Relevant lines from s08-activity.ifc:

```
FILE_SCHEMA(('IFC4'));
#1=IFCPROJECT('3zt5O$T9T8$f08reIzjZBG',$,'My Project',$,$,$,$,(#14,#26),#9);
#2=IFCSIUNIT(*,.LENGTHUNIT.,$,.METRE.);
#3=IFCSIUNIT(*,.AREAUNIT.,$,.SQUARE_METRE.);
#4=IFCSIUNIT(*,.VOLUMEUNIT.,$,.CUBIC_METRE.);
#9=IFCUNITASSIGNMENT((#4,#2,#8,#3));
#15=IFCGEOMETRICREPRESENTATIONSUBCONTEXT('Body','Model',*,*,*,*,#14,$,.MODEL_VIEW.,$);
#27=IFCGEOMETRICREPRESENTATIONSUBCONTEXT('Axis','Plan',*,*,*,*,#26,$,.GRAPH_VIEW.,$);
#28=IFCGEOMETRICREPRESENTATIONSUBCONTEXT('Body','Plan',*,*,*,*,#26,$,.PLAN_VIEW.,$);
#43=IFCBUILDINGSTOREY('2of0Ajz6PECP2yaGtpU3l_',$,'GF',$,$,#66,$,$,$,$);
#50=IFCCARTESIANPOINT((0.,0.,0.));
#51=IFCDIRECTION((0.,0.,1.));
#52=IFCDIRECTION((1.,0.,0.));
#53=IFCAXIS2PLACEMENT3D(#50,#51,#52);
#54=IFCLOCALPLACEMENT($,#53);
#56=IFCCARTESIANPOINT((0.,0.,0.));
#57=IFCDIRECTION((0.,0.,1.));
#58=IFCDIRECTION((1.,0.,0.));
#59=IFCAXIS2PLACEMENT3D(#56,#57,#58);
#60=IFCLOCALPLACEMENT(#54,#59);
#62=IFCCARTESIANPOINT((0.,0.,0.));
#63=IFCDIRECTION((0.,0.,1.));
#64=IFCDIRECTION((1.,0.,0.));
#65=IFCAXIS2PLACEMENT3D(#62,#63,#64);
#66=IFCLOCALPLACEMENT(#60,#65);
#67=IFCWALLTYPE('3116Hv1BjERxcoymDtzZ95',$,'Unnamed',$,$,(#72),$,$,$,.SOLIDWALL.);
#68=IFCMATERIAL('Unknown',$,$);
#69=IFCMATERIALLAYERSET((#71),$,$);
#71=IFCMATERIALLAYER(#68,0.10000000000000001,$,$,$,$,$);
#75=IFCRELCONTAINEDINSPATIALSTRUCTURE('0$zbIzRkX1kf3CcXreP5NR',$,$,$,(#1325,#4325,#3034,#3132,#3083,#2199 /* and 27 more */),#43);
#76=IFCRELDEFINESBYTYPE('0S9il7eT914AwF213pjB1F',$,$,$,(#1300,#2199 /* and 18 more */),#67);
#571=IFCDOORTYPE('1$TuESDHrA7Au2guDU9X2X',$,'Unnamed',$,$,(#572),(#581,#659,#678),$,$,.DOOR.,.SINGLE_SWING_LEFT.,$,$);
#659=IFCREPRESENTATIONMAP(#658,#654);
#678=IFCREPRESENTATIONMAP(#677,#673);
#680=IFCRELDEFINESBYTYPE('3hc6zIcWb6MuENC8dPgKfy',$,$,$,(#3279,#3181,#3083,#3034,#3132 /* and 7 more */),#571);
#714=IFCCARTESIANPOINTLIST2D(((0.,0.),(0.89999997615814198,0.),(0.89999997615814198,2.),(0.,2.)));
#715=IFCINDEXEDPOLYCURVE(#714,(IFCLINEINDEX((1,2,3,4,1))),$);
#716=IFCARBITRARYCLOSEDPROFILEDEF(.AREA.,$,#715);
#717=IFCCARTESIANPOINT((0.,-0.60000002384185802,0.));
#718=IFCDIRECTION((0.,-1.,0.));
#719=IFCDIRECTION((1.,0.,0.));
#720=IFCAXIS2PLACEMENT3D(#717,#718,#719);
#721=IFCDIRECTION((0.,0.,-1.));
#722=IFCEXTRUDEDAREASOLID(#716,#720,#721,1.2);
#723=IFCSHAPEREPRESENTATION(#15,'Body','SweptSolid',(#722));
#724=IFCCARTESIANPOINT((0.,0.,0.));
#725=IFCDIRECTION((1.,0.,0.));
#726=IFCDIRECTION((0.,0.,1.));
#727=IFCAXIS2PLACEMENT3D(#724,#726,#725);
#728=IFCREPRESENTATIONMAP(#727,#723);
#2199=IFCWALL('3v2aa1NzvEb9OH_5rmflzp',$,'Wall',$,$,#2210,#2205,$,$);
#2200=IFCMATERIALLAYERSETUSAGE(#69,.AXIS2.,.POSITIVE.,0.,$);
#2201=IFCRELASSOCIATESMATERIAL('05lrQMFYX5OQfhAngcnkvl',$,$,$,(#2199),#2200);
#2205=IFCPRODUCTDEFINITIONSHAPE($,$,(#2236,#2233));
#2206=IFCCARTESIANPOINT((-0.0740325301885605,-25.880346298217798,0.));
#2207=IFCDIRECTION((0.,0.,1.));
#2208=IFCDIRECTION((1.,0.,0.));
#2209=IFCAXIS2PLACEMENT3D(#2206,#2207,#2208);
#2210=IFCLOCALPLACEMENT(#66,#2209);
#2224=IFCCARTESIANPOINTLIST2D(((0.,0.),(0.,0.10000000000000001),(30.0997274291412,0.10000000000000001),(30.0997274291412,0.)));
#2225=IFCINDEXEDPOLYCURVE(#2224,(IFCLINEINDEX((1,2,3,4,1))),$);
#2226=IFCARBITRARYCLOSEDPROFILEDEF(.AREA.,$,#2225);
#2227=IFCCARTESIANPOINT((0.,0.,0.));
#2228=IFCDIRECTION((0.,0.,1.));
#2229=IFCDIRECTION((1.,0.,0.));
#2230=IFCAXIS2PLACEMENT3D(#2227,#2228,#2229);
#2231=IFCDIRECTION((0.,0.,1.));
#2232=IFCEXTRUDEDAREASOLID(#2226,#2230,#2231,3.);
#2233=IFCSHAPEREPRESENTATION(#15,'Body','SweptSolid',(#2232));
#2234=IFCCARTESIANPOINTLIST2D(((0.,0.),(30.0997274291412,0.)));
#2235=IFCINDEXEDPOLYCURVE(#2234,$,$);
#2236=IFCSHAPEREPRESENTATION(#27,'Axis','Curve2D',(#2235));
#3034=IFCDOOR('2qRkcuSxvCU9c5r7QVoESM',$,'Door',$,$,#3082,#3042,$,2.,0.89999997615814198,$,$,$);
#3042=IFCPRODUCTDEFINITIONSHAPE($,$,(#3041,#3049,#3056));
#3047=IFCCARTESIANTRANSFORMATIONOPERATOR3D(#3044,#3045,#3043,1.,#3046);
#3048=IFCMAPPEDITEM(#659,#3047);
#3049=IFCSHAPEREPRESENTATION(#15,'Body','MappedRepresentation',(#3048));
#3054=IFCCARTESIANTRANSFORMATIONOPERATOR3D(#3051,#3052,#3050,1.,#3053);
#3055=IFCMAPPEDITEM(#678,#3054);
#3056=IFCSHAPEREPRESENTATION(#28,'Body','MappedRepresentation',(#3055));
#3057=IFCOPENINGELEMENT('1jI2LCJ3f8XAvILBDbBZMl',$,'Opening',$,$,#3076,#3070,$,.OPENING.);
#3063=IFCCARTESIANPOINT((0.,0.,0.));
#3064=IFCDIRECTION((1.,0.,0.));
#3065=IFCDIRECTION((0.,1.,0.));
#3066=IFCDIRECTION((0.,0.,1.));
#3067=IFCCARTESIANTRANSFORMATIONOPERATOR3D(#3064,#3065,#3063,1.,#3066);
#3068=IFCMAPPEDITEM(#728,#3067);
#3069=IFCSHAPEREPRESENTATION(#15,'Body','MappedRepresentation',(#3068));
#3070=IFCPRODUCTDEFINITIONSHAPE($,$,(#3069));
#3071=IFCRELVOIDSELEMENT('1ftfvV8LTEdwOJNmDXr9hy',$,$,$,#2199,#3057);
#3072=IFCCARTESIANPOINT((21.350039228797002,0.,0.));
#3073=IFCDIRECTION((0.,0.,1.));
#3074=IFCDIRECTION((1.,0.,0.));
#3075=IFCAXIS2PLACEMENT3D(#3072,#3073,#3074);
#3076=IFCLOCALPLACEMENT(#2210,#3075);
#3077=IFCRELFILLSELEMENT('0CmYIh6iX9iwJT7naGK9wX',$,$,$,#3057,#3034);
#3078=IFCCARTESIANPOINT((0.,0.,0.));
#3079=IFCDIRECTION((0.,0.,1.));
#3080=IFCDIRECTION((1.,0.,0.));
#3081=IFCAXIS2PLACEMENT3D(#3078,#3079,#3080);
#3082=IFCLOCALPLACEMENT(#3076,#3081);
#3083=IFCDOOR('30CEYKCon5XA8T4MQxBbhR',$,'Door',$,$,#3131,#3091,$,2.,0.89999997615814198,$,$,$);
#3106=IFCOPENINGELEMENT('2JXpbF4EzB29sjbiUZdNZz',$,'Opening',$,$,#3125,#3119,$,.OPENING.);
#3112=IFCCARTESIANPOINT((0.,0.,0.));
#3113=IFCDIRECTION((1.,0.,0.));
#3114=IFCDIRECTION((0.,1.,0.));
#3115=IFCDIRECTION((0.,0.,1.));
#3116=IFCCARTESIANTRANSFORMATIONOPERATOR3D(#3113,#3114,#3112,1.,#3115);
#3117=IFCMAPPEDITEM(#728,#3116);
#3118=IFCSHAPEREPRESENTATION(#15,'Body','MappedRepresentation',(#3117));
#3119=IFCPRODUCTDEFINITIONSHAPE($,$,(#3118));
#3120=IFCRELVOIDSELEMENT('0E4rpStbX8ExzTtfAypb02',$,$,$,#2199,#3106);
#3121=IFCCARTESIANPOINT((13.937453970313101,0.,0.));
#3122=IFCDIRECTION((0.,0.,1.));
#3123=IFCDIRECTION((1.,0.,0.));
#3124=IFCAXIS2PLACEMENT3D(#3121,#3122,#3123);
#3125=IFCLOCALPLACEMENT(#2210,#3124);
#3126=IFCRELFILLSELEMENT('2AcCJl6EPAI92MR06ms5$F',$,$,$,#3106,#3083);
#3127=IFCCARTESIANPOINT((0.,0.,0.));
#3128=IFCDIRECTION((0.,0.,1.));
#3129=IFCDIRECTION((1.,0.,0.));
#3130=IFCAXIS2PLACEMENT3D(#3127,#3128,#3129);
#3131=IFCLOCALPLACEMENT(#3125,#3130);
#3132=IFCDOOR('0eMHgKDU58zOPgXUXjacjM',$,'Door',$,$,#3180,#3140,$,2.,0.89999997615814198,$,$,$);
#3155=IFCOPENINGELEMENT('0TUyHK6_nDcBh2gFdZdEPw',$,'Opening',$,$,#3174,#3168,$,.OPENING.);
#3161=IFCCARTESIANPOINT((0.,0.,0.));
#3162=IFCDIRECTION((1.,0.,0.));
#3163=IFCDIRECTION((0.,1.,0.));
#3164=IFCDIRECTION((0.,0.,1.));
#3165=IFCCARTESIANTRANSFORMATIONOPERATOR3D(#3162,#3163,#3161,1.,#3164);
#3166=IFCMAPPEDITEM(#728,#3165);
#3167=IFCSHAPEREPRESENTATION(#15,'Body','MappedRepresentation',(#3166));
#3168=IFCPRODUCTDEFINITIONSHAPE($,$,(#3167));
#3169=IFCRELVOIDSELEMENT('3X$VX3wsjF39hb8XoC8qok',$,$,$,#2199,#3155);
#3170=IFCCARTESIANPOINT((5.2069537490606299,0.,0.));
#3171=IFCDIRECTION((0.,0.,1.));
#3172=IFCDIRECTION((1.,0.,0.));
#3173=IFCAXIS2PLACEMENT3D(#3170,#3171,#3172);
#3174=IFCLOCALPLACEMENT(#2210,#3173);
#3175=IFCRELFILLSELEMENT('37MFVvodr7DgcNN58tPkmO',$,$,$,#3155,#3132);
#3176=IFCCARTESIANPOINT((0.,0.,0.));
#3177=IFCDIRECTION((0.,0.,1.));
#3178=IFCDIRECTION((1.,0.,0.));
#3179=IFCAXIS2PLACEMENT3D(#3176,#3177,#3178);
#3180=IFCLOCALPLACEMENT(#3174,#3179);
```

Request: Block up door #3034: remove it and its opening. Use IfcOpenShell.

```python
import ifcopenshell
import ifcopenshell.api.feature
import ifcopenshell.api.root
import ifcopenshell.geom
import ifcopenshell.util.shape

model = ifcopenshell.open("s08-activity.ifc")
settings = ifcopenshell.geom.settings()


def volume(element):
    """Net volume in cubic metres, openings subtracted."""
    shape = ifcopenshell.geom.create_shape(settings, element)
    return ifcopenshell.util.shape.get_volume(shape.geometry)


door = model.by_id(3034)
opening = door.FillsVoids[0].RelatingOpeningElement
wall = opening.VoidsElements[0].RelatingBuildingElement
before = volume(wall)

ifcopenshell.api.root.remove_product(model, product=door)
ifcopenshell.api.feature.remove_feature(model, feature=opening)

after = volume(wall)

print(f"wall volume {before:.3f} -> {after:.3f} m3")

model.write("s08-activity_updated.ifc")
```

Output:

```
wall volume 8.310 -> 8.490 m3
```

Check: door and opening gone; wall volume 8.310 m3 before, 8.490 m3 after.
